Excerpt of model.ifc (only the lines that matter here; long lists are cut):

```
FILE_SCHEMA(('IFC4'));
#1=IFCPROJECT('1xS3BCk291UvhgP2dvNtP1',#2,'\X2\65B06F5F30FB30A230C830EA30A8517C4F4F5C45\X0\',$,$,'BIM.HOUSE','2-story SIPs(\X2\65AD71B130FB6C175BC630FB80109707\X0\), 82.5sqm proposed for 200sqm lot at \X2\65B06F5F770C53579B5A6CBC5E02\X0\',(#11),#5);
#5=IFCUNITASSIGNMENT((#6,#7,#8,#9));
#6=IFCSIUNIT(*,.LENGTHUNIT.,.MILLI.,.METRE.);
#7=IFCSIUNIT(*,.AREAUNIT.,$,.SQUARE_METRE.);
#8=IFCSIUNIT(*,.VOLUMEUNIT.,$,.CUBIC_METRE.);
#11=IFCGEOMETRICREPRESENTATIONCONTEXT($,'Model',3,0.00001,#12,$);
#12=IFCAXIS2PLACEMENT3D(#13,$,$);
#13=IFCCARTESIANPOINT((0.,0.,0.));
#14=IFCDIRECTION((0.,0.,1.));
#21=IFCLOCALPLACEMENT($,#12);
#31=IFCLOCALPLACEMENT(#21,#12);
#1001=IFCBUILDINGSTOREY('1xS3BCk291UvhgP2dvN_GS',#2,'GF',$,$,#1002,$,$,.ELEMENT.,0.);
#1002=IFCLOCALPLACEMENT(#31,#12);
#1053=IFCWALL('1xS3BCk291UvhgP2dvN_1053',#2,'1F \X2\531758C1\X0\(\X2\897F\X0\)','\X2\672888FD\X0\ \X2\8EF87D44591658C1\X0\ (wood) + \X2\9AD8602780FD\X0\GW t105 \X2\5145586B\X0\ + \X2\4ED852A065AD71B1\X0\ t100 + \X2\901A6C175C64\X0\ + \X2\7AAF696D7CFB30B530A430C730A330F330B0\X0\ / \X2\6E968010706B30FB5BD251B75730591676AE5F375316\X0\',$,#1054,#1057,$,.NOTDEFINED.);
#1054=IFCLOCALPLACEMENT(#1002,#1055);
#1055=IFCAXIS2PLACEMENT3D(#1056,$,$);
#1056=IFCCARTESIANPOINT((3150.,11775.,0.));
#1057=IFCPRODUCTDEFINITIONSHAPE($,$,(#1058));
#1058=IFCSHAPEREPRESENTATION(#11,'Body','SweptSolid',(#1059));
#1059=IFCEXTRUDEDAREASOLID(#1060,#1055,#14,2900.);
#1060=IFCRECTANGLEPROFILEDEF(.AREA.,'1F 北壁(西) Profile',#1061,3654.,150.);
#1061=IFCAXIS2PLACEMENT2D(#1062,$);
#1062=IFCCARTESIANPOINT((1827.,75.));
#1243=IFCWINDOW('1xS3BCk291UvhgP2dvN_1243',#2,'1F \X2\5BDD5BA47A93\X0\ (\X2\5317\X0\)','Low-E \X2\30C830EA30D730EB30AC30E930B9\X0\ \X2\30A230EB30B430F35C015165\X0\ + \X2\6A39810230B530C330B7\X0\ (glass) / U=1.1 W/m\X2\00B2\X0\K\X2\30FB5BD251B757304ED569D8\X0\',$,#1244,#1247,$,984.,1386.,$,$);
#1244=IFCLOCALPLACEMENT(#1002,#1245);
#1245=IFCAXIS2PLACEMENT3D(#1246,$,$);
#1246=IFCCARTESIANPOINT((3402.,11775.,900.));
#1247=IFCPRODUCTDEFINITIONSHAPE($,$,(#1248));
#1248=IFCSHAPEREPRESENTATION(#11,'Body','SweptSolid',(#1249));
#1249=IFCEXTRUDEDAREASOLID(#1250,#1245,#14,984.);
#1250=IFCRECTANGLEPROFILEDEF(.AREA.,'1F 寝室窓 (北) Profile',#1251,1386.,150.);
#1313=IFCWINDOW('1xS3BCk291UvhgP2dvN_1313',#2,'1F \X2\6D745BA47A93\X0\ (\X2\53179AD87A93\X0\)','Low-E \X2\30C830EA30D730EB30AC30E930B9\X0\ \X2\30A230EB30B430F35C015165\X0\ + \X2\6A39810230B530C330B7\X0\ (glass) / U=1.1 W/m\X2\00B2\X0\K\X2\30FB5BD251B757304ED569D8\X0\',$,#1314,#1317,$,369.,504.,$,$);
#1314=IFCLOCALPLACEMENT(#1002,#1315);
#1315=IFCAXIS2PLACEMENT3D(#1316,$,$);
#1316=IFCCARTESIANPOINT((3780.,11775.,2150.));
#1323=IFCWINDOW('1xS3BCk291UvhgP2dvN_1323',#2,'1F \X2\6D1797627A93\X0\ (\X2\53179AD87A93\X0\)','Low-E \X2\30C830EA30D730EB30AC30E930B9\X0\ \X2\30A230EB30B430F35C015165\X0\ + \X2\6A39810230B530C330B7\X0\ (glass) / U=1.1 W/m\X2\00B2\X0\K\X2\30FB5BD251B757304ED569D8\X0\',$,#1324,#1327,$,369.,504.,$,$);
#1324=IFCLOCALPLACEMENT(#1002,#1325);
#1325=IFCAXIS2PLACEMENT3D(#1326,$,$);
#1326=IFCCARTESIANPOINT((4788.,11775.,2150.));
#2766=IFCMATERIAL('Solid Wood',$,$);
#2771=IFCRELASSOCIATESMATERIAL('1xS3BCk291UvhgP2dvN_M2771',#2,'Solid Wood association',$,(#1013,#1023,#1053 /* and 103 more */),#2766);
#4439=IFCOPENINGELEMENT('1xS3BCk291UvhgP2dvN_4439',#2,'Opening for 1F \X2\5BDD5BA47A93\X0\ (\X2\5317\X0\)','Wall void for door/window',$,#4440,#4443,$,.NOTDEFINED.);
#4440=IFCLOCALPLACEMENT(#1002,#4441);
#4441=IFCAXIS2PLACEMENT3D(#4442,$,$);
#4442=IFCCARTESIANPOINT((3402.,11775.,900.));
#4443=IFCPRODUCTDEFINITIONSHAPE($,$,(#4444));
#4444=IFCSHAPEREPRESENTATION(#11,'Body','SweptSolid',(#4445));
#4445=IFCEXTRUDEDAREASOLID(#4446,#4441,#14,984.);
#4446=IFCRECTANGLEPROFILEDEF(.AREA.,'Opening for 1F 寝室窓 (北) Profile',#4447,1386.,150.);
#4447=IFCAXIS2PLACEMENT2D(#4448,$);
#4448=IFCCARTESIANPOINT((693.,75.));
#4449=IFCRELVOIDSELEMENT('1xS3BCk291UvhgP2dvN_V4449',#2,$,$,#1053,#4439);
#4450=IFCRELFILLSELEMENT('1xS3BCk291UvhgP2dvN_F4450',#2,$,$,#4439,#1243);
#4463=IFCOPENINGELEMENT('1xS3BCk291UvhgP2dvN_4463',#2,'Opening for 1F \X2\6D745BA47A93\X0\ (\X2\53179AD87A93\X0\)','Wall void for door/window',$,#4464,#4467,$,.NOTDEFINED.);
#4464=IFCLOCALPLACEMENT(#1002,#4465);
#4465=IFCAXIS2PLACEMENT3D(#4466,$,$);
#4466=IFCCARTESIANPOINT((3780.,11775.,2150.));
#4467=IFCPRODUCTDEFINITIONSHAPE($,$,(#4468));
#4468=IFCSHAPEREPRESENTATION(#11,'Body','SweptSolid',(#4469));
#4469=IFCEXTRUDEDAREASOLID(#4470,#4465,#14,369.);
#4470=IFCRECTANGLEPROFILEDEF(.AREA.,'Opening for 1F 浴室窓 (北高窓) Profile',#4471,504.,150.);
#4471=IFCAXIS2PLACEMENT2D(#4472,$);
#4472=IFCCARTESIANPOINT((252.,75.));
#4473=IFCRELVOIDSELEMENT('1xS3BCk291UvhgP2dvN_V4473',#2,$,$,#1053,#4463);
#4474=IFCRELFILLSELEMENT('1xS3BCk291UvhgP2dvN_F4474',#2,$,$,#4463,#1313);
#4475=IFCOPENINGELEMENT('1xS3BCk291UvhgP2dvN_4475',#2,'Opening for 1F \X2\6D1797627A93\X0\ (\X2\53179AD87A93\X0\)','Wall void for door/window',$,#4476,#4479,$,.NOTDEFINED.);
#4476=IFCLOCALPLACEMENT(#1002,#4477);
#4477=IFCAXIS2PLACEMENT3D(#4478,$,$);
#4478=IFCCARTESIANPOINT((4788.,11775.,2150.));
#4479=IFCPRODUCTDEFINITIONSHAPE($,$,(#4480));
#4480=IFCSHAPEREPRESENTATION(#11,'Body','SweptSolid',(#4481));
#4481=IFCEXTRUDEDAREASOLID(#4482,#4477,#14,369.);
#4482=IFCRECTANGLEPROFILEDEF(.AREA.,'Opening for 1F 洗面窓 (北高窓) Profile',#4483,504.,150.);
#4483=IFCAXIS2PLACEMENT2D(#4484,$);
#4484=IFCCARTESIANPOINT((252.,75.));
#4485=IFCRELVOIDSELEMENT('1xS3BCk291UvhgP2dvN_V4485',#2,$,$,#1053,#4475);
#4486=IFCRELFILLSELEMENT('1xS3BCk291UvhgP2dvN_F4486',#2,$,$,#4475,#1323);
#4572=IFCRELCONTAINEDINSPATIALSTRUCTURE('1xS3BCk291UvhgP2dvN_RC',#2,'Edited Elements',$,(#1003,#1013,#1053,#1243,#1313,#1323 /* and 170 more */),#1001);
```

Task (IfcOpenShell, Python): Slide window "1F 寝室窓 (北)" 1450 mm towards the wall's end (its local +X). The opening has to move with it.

```python
import ifcopenshell
import ifcopenshell.api.geometry
import ifcopenshell.util.placement

model = ifcopenshell.open("model.ifc")

window = model.by_guid("1xS3BCk291UvhgP2dvN_1243")
opening = window.FillsVoids[0].RelatingOpeningElement
wall = opening.VoidsElements[0].RelatingBuildingElement

wall_matrix = ifcopenshell.util.placement.get_local_placement(wall.ObjectPlacement)
shift = wall_matrix[:3, 0] * 1450.0
before = ifcopenshell.util.placement.get_local_placement(window.ObjectPlacement)[:3, 3].copy()

# The window is not placed relative to its opening, so move both.
for product in (opening, window):
    matrix = ifcopenshell.util.placement.get_local_placement(product.ObjectPlacement)
    matrix[:3, 3] += shift
    ifcopenshell.api.geometry.edit_object_placement(model, product=product, matrix=matrix, is_si=False)

after = ifcopenshell.util.placement.get_local_placement(window.ObjectPlacement)[:3, 3]
print("window moved by", (after - before).round(3) + 0.0)

model.write("model_rev.ifc")
```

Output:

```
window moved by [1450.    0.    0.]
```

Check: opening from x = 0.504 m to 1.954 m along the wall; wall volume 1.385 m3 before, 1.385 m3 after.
